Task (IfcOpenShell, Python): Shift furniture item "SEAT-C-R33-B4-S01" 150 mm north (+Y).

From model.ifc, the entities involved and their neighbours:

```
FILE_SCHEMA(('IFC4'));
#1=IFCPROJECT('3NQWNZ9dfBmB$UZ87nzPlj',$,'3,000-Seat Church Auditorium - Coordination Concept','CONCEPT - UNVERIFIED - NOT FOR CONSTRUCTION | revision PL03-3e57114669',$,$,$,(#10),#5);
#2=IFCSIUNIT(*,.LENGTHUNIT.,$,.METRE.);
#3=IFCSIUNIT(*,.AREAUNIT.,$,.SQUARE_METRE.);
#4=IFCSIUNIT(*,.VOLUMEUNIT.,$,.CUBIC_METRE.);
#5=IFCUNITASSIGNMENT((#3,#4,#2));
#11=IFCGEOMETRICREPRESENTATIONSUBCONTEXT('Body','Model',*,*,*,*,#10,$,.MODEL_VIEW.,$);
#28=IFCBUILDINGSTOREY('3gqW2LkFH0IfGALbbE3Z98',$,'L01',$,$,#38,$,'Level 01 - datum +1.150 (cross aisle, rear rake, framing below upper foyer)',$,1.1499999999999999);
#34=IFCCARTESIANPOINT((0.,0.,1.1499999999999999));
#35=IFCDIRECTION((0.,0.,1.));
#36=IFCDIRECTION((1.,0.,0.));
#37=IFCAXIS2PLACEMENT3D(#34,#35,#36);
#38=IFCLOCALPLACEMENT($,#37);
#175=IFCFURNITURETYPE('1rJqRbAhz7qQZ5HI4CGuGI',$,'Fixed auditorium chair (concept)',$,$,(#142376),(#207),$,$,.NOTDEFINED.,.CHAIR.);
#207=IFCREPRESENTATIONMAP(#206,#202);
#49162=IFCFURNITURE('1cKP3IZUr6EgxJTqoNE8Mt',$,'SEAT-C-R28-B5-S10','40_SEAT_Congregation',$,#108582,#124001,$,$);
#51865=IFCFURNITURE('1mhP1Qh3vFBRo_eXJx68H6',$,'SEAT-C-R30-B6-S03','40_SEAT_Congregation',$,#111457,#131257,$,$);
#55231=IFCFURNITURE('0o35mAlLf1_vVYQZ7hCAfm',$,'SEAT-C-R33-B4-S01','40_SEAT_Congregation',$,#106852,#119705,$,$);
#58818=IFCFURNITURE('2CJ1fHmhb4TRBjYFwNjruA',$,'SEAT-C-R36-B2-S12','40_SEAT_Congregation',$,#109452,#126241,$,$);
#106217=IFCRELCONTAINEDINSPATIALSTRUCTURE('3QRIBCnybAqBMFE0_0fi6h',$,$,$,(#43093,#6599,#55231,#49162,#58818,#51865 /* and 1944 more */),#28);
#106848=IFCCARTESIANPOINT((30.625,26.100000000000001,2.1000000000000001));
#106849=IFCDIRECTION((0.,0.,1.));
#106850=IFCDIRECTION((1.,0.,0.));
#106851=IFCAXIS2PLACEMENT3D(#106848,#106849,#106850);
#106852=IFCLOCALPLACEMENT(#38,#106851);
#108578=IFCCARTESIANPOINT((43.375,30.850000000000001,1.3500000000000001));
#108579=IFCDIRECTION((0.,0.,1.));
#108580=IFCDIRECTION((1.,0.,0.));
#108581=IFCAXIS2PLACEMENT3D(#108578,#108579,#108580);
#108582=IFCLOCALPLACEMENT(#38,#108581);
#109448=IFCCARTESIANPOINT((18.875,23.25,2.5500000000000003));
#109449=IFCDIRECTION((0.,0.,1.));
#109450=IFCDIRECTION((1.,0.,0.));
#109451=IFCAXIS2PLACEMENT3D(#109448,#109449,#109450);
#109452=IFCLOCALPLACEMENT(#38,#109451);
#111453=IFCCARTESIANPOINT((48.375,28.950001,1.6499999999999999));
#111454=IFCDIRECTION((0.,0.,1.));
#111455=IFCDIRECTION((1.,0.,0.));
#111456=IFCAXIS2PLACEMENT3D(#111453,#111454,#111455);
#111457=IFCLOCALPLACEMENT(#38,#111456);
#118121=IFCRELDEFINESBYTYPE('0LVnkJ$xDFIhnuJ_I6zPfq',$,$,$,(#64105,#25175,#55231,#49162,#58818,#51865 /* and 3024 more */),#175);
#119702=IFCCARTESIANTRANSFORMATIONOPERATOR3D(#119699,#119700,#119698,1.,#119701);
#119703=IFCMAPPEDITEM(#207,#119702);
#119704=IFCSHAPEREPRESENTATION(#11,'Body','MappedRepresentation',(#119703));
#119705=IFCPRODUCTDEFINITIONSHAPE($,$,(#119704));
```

```python
import ifcopenshell
import ifcopenshell.api.geometry
import ifcopenshell.util.placement
import ifcopenshell.util.unit

model = ifcopenshell.open("model.ifc")
unit_scale = ifcopenshell.util.unit.calculate_unit_scale(model)

item = model.by_guid("0o35mAlLf1_vVYQZ7hCAfm")
matrix = ifcopenshell.util.placement.get_local_placement(item.ObjectPlacement)
matrix[1, 3] += 0.15 / unit_scale
ifcopenshell.api.geometry.edit_object_placement(model, product=item, matrix=matrix, is_si=False)

print(ifcopenshell.util.placement.get_local_placement(item.ObjectPlacement).round(3) + 0.0)

model.write("model_edited.ifc")
```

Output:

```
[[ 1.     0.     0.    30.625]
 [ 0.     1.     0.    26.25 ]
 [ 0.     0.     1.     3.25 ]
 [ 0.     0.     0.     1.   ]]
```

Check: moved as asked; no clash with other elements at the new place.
